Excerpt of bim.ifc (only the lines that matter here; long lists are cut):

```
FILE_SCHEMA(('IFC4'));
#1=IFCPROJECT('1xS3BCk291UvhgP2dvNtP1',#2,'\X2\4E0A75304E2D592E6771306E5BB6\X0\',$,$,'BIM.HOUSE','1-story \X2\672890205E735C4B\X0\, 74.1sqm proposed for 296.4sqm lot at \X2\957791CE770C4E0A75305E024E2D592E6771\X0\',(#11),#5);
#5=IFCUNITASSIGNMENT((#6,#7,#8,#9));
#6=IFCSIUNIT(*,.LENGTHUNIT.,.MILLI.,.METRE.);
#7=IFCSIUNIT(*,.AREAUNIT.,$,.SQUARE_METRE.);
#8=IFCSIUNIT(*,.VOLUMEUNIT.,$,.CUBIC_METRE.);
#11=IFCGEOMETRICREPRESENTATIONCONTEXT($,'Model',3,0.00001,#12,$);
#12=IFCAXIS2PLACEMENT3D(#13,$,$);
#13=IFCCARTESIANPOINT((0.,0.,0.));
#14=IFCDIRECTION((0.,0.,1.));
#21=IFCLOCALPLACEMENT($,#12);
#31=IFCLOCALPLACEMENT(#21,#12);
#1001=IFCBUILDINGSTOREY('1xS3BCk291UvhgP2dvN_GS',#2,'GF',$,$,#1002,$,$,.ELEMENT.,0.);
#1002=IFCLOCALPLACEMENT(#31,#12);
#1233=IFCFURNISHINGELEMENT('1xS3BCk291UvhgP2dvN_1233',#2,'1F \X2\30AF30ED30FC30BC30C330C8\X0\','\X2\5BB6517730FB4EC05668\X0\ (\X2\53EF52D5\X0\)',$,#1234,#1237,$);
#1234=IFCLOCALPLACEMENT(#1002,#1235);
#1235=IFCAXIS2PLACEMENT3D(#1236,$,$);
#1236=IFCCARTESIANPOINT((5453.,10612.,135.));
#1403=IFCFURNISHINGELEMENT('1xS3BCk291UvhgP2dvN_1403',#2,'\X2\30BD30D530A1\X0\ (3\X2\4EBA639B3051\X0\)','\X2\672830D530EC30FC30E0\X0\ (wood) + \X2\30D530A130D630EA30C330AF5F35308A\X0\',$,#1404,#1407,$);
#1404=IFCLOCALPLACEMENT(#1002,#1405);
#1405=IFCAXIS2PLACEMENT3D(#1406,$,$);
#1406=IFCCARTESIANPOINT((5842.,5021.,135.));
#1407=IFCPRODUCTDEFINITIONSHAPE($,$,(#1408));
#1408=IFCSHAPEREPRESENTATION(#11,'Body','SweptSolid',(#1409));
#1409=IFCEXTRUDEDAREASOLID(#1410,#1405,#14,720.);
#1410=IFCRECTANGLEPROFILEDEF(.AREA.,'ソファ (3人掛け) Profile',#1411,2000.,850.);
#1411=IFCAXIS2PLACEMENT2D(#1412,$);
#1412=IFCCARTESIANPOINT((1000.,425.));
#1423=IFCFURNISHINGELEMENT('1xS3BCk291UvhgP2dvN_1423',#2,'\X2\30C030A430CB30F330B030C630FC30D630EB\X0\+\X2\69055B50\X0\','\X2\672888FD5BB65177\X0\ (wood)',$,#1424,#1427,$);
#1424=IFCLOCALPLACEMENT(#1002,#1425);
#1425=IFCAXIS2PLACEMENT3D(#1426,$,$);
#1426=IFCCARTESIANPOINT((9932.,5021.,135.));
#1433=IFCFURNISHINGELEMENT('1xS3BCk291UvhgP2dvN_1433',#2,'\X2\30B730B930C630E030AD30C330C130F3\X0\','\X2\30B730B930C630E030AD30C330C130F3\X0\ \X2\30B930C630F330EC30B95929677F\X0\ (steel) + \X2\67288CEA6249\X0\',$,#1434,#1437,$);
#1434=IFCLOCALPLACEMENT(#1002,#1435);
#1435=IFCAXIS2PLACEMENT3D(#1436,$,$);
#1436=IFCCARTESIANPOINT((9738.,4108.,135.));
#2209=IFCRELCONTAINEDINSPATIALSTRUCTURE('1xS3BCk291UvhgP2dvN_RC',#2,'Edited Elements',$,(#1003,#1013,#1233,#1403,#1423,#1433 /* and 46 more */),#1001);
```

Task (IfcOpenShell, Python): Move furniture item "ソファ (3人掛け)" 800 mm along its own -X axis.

```python
import ifcopenshell
import ifcopenshell.api.geometry
import ifcopenshell.util.placement

model = ifcopenshell.open("bim.ifc")

item = model.by_id(1403)
matrix = ifcopenshell.util.placement.get_local_placement(item.ObjectPlacement)
matrix[:3, 3] -= matrix[:3, 0] * 800.0
ifcopenshell.api.geometry.edit_object_placement(model, product=item, matrix=matrix, is_si=False)

print(ifcopenshell.util.placement.get_local_placement(item.ObjectPlacement).round(3) + 0.0)

model.write("bim-out.ifc")
```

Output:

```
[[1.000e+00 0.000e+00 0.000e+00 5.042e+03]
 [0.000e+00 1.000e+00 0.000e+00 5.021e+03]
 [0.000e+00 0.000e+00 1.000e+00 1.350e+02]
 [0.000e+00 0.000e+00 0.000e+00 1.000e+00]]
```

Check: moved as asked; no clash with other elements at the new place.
